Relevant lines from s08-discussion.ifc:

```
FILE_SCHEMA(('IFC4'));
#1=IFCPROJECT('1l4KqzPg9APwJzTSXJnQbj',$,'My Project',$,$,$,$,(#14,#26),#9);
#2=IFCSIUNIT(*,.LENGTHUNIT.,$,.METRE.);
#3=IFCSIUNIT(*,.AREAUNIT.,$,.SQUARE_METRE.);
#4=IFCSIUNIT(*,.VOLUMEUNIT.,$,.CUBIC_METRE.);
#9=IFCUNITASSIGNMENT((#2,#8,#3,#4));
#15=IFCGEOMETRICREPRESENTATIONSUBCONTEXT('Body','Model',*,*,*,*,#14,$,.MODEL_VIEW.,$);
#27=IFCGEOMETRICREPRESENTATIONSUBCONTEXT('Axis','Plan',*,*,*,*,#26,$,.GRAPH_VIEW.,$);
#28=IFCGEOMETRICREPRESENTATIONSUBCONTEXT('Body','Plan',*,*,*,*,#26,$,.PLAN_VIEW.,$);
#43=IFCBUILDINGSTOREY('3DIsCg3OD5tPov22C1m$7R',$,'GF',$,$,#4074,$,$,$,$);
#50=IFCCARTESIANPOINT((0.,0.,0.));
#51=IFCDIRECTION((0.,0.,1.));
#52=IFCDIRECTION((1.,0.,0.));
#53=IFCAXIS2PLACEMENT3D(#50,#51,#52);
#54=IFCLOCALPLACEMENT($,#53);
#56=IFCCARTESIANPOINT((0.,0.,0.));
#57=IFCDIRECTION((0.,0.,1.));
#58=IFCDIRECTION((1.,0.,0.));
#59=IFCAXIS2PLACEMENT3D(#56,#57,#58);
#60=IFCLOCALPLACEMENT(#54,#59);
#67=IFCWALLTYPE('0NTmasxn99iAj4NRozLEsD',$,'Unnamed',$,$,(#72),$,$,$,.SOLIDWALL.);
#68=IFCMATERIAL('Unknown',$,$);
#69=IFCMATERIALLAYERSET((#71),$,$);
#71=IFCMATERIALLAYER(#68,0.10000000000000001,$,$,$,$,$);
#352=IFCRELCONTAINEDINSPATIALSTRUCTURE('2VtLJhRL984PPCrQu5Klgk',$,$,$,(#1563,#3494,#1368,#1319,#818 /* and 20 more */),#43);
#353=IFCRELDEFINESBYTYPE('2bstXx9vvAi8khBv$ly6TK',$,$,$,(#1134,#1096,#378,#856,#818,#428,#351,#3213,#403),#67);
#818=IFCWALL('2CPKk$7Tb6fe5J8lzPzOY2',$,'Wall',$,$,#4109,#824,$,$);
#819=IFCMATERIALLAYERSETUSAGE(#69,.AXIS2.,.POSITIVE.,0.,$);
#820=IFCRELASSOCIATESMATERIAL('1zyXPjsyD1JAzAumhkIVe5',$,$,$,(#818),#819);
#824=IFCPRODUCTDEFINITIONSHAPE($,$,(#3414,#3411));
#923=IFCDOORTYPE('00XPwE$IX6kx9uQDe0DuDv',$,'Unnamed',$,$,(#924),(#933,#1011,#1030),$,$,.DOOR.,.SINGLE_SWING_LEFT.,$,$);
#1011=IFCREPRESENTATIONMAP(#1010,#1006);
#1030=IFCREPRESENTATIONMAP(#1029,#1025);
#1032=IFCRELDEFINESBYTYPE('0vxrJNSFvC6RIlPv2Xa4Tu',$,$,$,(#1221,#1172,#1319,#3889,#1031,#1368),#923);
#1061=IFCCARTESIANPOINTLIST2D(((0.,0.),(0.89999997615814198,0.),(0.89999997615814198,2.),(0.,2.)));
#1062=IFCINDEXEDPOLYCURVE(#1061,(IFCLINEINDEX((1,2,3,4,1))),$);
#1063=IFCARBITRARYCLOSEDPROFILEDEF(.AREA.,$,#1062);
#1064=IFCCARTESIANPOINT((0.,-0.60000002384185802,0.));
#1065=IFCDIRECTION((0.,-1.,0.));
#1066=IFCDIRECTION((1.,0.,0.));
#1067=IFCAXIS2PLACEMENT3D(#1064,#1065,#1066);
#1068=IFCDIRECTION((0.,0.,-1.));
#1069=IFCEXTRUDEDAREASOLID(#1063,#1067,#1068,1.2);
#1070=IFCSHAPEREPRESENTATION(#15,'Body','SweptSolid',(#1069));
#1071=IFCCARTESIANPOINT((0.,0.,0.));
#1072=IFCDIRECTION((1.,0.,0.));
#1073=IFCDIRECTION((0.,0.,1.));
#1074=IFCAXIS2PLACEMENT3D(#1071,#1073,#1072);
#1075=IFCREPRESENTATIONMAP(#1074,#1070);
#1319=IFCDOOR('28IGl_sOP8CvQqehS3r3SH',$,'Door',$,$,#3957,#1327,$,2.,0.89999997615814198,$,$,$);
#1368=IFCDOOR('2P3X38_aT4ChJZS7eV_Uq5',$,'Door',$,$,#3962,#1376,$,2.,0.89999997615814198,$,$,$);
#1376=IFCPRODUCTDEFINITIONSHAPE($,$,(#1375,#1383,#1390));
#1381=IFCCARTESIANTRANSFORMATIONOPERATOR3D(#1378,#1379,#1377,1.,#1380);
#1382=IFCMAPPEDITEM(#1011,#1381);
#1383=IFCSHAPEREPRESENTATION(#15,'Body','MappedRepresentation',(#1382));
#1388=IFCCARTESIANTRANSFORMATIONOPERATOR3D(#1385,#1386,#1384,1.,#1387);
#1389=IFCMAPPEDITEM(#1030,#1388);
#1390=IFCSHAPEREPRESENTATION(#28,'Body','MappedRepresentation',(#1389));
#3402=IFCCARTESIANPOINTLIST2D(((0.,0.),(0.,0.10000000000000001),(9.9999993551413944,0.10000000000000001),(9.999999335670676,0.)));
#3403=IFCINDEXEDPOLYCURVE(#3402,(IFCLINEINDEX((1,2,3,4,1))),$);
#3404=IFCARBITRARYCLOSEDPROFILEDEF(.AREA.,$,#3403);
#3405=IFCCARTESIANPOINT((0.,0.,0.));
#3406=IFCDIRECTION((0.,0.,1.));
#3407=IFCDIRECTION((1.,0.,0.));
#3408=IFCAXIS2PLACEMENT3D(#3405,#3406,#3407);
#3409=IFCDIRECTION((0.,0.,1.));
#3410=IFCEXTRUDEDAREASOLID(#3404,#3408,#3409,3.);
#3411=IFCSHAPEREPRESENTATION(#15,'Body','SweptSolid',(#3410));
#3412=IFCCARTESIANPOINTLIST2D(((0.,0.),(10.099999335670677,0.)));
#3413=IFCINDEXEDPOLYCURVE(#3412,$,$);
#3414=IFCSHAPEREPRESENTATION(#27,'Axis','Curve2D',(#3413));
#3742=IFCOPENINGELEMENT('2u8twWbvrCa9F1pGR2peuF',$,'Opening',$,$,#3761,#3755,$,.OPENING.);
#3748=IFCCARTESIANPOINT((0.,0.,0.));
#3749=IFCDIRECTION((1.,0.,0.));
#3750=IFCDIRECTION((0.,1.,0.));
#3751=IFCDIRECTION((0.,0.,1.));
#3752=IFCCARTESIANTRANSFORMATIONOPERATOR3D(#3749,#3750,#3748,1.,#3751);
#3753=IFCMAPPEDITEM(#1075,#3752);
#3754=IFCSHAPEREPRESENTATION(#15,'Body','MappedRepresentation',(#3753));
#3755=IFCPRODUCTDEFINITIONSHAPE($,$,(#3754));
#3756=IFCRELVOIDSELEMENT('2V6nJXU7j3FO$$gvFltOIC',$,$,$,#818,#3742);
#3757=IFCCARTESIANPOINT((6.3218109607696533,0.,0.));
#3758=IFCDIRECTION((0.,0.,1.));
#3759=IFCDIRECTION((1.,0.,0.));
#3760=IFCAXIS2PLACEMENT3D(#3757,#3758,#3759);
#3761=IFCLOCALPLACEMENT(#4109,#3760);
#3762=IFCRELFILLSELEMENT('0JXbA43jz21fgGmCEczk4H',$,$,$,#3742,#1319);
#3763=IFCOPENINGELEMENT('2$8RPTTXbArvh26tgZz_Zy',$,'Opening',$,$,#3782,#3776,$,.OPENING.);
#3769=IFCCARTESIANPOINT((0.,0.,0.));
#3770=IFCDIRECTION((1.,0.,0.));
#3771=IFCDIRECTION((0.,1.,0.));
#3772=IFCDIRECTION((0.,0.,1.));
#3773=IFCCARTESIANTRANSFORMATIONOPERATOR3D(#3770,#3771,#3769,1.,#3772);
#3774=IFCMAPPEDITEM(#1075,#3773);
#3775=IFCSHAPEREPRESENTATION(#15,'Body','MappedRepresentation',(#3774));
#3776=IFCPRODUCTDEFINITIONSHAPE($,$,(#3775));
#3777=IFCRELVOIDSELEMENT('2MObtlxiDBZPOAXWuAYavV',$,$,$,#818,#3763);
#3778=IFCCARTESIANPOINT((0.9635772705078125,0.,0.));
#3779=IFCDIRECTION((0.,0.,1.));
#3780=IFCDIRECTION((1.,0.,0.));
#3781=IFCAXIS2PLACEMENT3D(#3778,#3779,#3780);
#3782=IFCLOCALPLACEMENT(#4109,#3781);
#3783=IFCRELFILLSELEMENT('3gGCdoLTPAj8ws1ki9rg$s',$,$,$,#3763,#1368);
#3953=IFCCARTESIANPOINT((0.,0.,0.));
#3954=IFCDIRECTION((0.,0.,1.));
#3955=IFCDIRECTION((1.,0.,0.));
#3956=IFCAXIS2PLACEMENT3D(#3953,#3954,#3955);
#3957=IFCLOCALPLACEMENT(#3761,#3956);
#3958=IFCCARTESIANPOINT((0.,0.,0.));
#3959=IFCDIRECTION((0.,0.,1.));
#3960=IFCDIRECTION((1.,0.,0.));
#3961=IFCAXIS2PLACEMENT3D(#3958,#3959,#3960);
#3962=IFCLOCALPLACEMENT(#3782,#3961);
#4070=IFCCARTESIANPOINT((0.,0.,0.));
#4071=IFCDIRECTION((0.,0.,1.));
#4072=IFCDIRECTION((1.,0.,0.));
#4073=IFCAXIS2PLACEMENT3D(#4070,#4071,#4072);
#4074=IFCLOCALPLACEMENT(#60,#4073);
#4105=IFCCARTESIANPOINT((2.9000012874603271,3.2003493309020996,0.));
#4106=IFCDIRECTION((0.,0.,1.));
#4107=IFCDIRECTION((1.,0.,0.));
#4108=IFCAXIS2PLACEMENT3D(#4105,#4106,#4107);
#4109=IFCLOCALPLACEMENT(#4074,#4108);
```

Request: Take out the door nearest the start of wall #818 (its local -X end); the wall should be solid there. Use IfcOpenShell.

```python
import ifcopenshell
import ifcopenshell.api.feature
import ifcopenshell.api.root
import ifcopenshell.geom
import ifcopenshell.util.shape

model = ifcopenshell.open("s08-discussion.ifc")
settings = ifcopenshell.geom.settings()


def volume(element):
    """Net volume in cubic metres, openings subtracted."""
    shape = ifcopenshell.geom.create_shape(settings, element)
    return ifcopenshell.util.shape.get_volume(shape.geometry)


door = model.by_guid("2P3X38_aT4ChJZS7eV_Uq5")
opening = door.FillsVoids[0].RelatingOpeningElement
wall = opening.VoidsElements[0].RelatingBuildingElement
before = volume(wall)

ifcopenshell.api.root.remove_product(model, product=door)
ifcopenshell.api.feature.remove_feature(model, feature=opening)

after = volume(wall)

print(f"wall volume {before:.3f} -> {after:.3f} m3")

model.write("s08-discussion_rev.ifc")
```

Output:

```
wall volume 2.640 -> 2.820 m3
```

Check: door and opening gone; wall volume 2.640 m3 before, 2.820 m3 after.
